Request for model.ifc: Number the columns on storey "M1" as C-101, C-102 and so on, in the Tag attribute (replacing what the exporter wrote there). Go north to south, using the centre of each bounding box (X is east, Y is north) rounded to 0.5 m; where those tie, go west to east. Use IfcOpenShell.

First a look at what the model holds.

```python
import ifcopenshell
import ifcopenshell.util.element
import ifcopenshell.util.placement

model = ifcopenshell.open("model.ifc")
print(model.schema)
storey = next(s for s in model.by_type("IfcBuildingStorey") if s.Name == "M1")
columns = [e for e in ifcopenshell.util.element.get_decomposition(storey) if e.is_a("IfcColumn")]
for e in sorted(columns, key=lambda e: e.id()):
    origin = ifcopenshell.util.placement.get_local_placement(e.ObjectPlacement)[:3, 3]
    print(e.id(), e.Tag, e.Name, origin.round(2) + 0.0, sep=" | ")
```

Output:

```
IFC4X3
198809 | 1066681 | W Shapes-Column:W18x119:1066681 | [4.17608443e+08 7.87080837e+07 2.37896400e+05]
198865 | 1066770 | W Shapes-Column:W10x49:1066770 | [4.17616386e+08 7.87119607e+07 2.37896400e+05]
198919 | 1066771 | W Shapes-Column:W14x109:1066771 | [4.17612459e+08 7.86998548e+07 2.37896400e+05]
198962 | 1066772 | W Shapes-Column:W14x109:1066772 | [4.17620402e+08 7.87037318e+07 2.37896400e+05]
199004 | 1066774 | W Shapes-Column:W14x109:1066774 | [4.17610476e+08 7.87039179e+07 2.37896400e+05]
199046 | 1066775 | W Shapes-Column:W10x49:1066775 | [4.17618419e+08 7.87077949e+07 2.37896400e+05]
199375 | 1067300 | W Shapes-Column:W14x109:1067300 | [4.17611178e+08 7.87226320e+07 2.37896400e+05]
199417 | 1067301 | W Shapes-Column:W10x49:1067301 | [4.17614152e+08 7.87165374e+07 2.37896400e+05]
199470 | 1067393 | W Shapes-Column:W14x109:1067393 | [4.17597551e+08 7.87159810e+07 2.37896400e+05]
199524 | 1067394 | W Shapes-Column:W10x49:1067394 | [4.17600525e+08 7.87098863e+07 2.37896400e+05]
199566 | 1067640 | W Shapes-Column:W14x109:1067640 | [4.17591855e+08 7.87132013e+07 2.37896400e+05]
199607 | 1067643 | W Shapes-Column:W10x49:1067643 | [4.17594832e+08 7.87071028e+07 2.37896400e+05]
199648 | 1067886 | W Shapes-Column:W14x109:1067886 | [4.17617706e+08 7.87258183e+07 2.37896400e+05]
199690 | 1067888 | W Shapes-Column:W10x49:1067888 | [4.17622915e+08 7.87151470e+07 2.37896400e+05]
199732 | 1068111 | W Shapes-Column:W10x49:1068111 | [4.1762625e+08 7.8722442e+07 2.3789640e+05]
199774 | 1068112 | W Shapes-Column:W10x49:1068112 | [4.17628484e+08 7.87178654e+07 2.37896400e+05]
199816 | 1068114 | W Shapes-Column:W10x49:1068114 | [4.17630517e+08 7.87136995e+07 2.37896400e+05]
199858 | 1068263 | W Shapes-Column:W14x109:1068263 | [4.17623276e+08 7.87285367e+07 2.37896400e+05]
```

```python
import ifcopenshell
import ifcopenshell.geom
import ifcopenshell.util.element
import ifcopenshell.util.shape

model = ifcopenshell.open("model.ifc")
settings = ifcopenshell.geom.settings()
settings.set("use-world-coords", True)


def centre(element):
    shape = ifcopenshell.geom.create_shape(settings, element)
    return ifcopenshell.util.shape.get_bbox_centroid(shape.geometry)


storey = next(s for s in model.by_type("IfcBuildingStorey") if s.Name == "M1")
columns = [e for e in ifcopenshell.util.element.get_decomposition(storey) if e.is_a("IfcColumn")]

# Insertion points can sit at a corner or the storey origin, so sort by the geometry (in metres).
centres = {e: centre(e) for e in columns}
columns.sort(key=lambda e: (-round(centres[e][1] / 0.5), centres[e][0]))

for i, e in enumerate(columns, start=1):
    number = f"C-1{i:02d}"
    e.Tag = number
    print(e.id(), number)

model.write("model_updated.ifc")
```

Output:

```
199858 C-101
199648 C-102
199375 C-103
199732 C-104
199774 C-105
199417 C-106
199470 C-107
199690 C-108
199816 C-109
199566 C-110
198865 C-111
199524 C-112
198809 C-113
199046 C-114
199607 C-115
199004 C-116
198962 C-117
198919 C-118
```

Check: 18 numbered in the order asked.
